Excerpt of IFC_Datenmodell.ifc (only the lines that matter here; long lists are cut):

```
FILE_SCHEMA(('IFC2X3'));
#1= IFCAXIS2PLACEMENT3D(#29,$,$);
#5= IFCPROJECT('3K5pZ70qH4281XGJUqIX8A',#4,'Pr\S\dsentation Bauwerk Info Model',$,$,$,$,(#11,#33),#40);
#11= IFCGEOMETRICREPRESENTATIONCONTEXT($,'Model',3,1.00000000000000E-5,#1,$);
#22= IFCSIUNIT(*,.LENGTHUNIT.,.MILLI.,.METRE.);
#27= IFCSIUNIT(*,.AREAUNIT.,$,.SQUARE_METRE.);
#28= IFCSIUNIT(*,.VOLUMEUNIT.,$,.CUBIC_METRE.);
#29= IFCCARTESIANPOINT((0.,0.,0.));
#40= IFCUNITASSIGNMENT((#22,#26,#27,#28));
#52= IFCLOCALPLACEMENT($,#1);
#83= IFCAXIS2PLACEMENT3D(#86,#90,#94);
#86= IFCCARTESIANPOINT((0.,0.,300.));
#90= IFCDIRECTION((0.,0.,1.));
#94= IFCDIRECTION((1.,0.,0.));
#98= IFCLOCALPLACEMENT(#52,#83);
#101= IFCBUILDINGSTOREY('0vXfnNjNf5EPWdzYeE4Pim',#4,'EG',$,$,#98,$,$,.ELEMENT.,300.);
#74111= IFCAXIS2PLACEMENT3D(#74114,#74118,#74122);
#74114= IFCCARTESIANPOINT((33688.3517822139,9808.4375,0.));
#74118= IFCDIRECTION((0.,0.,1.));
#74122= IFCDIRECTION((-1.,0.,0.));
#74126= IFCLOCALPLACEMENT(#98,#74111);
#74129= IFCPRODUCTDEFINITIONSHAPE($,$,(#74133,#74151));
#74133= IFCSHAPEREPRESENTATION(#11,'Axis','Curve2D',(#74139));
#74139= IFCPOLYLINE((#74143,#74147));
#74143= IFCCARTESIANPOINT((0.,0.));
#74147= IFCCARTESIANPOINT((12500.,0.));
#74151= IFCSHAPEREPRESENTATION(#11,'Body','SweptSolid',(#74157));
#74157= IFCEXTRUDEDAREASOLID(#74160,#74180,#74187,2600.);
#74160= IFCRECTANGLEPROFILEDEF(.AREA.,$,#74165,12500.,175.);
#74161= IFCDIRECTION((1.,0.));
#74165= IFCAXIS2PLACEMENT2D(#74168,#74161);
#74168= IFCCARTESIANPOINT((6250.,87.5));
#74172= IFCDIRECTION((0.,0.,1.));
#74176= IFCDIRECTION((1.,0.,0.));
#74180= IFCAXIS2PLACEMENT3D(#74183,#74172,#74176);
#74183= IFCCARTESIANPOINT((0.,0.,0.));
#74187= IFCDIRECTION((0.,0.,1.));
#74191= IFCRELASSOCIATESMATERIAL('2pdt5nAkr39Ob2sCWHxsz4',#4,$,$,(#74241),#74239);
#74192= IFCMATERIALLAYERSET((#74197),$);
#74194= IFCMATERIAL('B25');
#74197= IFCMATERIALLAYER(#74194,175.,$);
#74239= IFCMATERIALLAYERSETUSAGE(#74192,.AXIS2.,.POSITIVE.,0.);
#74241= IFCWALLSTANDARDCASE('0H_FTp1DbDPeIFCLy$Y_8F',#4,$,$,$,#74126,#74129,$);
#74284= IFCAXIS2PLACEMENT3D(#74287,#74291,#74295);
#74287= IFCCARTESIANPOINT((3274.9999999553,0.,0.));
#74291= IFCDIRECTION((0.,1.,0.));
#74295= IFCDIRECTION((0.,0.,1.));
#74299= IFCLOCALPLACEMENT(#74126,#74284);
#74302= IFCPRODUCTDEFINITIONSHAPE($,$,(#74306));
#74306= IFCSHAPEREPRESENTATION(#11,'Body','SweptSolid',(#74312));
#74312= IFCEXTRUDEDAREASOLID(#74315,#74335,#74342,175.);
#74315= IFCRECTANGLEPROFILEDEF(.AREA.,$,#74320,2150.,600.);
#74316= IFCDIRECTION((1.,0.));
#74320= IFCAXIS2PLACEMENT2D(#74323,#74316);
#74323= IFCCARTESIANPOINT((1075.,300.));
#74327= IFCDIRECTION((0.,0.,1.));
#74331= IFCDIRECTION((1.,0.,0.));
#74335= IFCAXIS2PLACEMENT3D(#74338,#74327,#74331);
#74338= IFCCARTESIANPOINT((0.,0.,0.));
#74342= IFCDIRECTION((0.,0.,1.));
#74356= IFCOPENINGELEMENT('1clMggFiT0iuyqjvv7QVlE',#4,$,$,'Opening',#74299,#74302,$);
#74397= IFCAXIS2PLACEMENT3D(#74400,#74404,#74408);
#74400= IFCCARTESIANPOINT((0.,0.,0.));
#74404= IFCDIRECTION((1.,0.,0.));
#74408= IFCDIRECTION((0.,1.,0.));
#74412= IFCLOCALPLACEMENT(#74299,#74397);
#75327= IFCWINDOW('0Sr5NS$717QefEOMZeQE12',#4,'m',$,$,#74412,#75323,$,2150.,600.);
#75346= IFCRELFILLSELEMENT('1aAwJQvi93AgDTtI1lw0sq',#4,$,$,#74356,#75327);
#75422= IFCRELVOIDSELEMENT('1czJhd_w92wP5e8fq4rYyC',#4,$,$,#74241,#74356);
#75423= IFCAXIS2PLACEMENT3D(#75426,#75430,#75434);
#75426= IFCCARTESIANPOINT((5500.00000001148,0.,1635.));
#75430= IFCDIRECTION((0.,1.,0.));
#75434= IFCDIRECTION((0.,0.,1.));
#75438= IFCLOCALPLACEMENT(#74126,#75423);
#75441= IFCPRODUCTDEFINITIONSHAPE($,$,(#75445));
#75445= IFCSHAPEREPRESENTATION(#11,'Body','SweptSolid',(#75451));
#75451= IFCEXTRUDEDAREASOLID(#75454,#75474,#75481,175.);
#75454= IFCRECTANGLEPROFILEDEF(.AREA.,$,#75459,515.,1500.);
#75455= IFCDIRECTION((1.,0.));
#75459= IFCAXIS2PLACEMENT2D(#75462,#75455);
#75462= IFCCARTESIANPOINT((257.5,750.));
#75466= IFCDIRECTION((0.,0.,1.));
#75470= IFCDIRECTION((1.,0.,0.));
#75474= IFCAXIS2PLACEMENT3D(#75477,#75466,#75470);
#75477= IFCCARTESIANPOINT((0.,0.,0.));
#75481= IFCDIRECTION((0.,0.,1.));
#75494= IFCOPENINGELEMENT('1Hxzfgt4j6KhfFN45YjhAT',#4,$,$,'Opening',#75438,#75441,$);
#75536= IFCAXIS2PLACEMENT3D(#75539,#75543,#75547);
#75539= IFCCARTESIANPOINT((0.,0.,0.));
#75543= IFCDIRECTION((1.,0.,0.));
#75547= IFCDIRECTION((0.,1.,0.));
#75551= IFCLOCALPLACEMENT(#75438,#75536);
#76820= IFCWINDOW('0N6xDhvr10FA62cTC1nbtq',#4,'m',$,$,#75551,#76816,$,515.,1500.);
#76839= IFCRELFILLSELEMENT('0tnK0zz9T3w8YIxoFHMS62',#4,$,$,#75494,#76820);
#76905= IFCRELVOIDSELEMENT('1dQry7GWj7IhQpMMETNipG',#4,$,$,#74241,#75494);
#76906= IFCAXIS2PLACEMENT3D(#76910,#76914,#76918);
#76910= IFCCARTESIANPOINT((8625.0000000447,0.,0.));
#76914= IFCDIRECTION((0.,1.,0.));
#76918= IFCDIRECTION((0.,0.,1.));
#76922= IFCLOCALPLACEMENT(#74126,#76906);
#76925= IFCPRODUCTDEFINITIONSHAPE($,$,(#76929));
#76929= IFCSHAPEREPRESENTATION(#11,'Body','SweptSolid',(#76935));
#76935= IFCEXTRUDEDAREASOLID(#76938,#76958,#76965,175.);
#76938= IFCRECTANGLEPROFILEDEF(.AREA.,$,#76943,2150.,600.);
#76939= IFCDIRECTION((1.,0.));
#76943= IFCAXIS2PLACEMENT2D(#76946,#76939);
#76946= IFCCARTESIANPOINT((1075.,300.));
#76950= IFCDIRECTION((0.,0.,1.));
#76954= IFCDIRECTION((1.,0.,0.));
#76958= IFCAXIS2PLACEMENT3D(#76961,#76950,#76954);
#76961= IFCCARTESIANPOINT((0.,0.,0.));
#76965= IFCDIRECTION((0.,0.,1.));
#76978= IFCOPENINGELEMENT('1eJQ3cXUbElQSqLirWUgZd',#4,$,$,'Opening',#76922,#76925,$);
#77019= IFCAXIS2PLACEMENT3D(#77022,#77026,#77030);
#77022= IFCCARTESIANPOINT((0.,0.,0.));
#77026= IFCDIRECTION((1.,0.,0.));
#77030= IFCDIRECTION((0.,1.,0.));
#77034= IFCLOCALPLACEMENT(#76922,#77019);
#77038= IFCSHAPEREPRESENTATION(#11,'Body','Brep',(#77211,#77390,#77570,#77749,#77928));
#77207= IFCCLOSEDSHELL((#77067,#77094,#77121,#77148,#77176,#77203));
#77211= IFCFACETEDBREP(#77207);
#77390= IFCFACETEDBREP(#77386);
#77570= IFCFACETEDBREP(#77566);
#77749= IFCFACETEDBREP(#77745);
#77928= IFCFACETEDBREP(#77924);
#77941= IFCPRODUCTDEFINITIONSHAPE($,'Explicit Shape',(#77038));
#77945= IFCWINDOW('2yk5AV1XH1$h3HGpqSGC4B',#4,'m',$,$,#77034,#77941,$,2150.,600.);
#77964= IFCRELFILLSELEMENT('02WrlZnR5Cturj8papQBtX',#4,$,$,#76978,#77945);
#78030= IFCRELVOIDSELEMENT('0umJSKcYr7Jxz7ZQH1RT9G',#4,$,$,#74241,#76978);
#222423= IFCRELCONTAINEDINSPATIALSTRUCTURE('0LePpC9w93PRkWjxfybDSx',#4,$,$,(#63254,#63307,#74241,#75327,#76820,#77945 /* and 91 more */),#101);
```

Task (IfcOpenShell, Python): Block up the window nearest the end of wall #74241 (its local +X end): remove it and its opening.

```python
import ifcopenshell
import ifcopenshell.api.feature
import ifcopenshell.api.root
import ifcopenshell.geom
import ifcopenshell.util.shape

model = ifcopenshell.open("IFC_Datenmodell.ifc")
settings = ifcopenshell.geom.settings()


def volume(element):
    """Net volume in cubic metres, openings subtracted."""
    shape = ifcopenshell.geom.create_shape(settings, element)
    return ifcopenshell.util.shape.get_volume(shape.geometry)


window = model.by_guid("2yk5AV1XH1$h3HGpqSGC4B")
opening = window.FillsVoids[0].RelatingOpeningElement
wall = opening.VoidsElements[0].RelatingBuildingElement
before = volume(wall)

ifcopenshell.api.root.remove_product(model, product=window)
ifcopenshell.api.feature.remove_feature(model, feature=opening)

after = volume(wall)

print(f"wall volume {before:.3f} -> {after:.3f} m3")

model.write("IFC_Datenmodell_updated.ifc")
```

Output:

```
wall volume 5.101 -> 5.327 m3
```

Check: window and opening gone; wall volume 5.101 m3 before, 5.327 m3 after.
